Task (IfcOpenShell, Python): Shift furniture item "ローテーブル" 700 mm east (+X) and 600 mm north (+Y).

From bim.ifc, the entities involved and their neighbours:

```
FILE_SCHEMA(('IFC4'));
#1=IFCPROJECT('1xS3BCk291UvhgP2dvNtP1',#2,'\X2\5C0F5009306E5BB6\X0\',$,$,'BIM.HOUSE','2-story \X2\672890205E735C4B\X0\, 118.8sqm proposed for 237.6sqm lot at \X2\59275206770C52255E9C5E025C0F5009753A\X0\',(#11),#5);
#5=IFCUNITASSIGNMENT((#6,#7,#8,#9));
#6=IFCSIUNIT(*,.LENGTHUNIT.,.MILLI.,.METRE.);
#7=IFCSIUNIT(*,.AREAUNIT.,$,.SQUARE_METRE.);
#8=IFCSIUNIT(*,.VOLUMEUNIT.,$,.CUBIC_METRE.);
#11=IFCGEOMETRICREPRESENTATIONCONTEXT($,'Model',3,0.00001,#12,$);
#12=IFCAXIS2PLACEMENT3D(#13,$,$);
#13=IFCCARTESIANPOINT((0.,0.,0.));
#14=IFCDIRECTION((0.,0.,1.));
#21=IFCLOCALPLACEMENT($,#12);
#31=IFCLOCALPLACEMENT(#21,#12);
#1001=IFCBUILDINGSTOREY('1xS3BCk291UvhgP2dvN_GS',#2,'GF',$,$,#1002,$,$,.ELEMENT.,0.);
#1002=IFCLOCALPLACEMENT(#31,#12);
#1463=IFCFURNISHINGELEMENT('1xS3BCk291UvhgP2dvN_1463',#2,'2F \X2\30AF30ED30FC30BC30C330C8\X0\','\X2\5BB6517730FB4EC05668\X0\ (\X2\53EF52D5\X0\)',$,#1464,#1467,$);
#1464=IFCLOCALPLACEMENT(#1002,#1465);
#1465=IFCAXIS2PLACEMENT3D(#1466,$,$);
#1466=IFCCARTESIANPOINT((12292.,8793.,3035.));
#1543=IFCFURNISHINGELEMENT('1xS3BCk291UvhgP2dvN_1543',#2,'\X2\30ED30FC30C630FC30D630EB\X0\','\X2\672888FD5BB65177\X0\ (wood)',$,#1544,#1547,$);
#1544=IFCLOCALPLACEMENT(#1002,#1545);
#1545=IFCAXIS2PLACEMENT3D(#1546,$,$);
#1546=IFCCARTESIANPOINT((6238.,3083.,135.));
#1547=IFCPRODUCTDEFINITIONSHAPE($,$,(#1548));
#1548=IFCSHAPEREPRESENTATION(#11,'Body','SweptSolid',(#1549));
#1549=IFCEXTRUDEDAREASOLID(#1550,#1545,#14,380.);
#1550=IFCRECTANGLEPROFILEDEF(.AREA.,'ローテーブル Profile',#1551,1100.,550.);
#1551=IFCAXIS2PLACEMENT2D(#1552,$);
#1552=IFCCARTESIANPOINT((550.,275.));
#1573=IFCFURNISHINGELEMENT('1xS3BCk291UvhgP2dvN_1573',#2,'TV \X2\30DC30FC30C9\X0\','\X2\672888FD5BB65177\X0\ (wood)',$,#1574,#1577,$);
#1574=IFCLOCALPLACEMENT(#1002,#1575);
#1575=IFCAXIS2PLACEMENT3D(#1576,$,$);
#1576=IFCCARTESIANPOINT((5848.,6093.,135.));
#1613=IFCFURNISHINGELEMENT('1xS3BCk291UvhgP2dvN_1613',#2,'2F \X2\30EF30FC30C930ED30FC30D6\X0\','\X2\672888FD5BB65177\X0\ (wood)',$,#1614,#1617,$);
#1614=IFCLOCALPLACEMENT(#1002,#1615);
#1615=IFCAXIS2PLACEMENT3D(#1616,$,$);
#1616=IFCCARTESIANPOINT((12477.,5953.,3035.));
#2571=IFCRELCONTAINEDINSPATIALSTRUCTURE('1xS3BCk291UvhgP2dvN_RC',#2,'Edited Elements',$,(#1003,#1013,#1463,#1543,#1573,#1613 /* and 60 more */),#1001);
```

```python
import ifcopenshell
import ifcopenshell.api.geometry
import ifcopenshell.util.placement
import ifcopenshell.util.unit

model = ifcopenshell.open("bim.ifc")
unit_scale = ifcopenshell.util.unit.calculate_unit_scale(model)

item = model.by_guid("1xS3BCk291UvhgP2dvN_1543")
matrix = ifcopenshell.util.placement.get_local_placement(item.ObjectPlacement)
matrix[0, 3] += 0.7 / unit_scale
matrix[1, 3] += 0.6 / unit_scale
ifcopenshell.api.geometry.edit_object_placement(model, product=item, matrix=matrix, is_si=False)

print(ifcopenshell.util.placement.get_local_placement(item.ObjectPlacement).round(3) + 0.0)

model.write("bim-out.ifc")
```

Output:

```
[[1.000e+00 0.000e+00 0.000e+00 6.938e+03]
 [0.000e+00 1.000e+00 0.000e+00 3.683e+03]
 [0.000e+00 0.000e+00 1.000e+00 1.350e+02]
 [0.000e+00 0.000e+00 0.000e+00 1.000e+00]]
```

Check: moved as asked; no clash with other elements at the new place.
